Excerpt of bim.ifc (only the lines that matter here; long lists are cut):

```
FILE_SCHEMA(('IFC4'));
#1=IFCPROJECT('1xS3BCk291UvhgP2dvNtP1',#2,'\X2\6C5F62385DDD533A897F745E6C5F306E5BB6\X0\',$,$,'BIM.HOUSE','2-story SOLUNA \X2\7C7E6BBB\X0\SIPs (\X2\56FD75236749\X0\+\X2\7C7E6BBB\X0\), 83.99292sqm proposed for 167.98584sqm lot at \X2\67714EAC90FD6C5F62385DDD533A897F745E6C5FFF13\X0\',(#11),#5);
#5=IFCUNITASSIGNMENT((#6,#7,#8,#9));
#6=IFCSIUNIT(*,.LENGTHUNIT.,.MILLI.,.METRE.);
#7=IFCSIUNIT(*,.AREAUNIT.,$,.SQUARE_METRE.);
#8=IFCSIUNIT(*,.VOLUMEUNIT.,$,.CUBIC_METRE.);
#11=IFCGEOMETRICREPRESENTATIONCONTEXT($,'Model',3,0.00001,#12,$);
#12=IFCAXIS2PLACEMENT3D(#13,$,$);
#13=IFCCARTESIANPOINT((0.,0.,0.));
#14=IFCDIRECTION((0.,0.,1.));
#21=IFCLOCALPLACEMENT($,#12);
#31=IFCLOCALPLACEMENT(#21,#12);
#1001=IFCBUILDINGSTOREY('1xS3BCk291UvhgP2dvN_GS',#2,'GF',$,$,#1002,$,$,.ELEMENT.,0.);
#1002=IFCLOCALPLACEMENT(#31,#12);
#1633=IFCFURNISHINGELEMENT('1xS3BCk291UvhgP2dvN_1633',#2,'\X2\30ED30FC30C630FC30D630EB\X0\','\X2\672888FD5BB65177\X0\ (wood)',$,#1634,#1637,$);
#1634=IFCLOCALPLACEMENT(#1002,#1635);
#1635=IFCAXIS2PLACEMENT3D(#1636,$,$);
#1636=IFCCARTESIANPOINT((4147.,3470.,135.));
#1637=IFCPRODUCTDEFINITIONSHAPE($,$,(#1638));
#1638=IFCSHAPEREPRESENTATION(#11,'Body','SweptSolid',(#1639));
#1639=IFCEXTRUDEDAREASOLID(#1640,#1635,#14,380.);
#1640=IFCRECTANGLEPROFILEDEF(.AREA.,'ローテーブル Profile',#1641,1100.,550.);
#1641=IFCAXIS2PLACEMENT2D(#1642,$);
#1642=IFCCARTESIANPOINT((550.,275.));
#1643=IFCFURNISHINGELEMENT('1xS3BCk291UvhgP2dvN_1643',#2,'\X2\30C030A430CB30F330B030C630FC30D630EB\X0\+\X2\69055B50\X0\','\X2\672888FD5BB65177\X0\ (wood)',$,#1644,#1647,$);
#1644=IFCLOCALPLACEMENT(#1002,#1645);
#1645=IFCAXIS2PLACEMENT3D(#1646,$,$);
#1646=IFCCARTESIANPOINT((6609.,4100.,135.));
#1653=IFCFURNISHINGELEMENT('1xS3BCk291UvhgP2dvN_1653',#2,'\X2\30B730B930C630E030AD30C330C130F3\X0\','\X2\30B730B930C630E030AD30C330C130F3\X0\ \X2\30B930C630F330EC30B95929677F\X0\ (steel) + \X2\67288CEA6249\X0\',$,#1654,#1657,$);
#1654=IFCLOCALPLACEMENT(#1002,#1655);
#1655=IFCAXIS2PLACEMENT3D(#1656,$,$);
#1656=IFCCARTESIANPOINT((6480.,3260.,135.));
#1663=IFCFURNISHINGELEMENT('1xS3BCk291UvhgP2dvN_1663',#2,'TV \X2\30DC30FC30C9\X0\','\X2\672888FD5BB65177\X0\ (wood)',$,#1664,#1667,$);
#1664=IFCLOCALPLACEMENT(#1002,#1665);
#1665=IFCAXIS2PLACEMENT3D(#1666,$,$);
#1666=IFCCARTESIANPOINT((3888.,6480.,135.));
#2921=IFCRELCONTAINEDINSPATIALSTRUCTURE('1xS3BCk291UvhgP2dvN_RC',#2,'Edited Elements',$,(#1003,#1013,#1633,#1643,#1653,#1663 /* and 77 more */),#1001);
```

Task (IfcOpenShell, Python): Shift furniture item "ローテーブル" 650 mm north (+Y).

```python
import ifcopenshell
import ifcopenshell.api.geometry
import ifcopenshell.util.placement
import ifcopenshell.util.unit

model = ifcopenshell.open("bim.ifc")
unit_scale = ifcopenshell.util.unit.calculate_unit_scale(model)

item = model.by_id(1633)
matrix = ifcopenshell.util.placement.get_local_placement(item.ObjectPlacement)
matrix[1, 3] += 0.65 / unit_scale
ifcopenshell.api.geometry.edit_object_placement(model, product=item, matrix=matrix, is_si=False)

print(ifcopenshell.util.placement.get_local_placement(item.ObjectPlacement).round(3) + 0.0)

model.write("bim-out.ifc")
```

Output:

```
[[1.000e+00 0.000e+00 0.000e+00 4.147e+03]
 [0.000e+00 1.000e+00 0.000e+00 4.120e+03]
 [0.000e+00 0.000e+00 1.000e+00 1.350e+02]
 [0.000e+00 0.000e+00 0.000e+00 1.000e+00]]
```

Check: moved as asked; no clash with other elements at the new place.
